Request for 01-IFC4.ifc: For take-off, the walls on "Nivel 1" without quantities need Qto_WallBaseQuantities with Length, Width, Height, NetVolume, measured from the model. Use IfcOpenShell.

First a look at what the model holds.

```python
import ifcopenshell
import ifcopenshell.util.element
import ifcopenshell.util.unit

model = ifcopenshell.open("01-IFC4.ifc")
print(model.schema)
for unit_type in ("LENGTHUNIT", "AREAUNIT", "VOLUMEUNIT"):
    print(unit_type, ifcopenshell.util.unit.calculate_unit_scale(model, unit_type))
storey = next(s for s in model.by_type("IfcBuildingStorey") if s.Name == "Nivel 1")
walls = [e for e in ifcopenshell.util.element.get_decomposition(storey) if e.is_a("IfcWall")]
for e in sorted(walls, key=lambda e: e.id()):
    print(e.id(), e.is_a(), e.Name, list(ifcopenshell.util.element.get_psets(e, qtos_only=True)), sep=" | ")
```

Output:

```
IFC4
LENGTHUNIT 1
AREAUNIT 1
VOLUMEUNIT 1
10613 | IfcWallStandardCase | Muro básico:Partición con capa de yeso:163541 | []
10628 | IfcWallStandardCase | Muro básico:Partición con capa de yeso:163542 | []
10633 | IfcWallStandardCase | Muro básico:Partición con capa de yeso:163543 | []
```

```python
import ifcopenshell
import ifcopenshell.api.pset
import ifcopenshell.geom
import ifcopenshell.util.element
import ifcopenshell.util.shape
import ifcopenshell.util.unit

model = ifcopenshell.open("01-IFC4.ifc")
unit_scale = ifcopenshell.util.unit.calculate_unit_scale(model)
volume_scale = ifcopenshell.util.unit.calculate_unit_scale(model, "VOLUMEUNIT")
settings = ifcopenshell.geom.settings()

storey = next(s for s in model.by_type("IfcBuildingStorey") if s.Name == "Nivel 1")
walls = [e for e in ifcopenshell.util.element.get_decomposition(storey) if e.is_a("IfcWall")]

for e in sorted(walls, key=lambda e: e.id()):
    if ifcopenshell.util.element.get_psets(e, qtos_only=True, should_inherit=False):
        continue
    # Geometry comes back in metres, in the element's own axes.
    shape = ifcopenshell.geom.create_shape(settings, e)
    values = {
        "Length": ifcopenshell.util.shape.get_x(shape.geometry) / unit_scale,
        "Width": ifcopenshell.util.shape.get_y(shape.geometry) / unit_scale,
        "Height": ifcopenshell.util.shape.get_z(shape.geometry) / unit_scale,
        "NetVolume": ifcopenshell.util.shape.get_volume(shape.geometry) / volume_scale,
    }
    qto = ifcopenshell.api.pset.add_qto(model, product=e, name="Qto_WallBaseQuantities")
    ifcopenshell.api.pset.edit_qto(model, qto=qto, properties=values)
    print(e.id(), {k: round(v, 3) for k, v in values.items()})

model.write("01-IFC4_edited.ifc")
```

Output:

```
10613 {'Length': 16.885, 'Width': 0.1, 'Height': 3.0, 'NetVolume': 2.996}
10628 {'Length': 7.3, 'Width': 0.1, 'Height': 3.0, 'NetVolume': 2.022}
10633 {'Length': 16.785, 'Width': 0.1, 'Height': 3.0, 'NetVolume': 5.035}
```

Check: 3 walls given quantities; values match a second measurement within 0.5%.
